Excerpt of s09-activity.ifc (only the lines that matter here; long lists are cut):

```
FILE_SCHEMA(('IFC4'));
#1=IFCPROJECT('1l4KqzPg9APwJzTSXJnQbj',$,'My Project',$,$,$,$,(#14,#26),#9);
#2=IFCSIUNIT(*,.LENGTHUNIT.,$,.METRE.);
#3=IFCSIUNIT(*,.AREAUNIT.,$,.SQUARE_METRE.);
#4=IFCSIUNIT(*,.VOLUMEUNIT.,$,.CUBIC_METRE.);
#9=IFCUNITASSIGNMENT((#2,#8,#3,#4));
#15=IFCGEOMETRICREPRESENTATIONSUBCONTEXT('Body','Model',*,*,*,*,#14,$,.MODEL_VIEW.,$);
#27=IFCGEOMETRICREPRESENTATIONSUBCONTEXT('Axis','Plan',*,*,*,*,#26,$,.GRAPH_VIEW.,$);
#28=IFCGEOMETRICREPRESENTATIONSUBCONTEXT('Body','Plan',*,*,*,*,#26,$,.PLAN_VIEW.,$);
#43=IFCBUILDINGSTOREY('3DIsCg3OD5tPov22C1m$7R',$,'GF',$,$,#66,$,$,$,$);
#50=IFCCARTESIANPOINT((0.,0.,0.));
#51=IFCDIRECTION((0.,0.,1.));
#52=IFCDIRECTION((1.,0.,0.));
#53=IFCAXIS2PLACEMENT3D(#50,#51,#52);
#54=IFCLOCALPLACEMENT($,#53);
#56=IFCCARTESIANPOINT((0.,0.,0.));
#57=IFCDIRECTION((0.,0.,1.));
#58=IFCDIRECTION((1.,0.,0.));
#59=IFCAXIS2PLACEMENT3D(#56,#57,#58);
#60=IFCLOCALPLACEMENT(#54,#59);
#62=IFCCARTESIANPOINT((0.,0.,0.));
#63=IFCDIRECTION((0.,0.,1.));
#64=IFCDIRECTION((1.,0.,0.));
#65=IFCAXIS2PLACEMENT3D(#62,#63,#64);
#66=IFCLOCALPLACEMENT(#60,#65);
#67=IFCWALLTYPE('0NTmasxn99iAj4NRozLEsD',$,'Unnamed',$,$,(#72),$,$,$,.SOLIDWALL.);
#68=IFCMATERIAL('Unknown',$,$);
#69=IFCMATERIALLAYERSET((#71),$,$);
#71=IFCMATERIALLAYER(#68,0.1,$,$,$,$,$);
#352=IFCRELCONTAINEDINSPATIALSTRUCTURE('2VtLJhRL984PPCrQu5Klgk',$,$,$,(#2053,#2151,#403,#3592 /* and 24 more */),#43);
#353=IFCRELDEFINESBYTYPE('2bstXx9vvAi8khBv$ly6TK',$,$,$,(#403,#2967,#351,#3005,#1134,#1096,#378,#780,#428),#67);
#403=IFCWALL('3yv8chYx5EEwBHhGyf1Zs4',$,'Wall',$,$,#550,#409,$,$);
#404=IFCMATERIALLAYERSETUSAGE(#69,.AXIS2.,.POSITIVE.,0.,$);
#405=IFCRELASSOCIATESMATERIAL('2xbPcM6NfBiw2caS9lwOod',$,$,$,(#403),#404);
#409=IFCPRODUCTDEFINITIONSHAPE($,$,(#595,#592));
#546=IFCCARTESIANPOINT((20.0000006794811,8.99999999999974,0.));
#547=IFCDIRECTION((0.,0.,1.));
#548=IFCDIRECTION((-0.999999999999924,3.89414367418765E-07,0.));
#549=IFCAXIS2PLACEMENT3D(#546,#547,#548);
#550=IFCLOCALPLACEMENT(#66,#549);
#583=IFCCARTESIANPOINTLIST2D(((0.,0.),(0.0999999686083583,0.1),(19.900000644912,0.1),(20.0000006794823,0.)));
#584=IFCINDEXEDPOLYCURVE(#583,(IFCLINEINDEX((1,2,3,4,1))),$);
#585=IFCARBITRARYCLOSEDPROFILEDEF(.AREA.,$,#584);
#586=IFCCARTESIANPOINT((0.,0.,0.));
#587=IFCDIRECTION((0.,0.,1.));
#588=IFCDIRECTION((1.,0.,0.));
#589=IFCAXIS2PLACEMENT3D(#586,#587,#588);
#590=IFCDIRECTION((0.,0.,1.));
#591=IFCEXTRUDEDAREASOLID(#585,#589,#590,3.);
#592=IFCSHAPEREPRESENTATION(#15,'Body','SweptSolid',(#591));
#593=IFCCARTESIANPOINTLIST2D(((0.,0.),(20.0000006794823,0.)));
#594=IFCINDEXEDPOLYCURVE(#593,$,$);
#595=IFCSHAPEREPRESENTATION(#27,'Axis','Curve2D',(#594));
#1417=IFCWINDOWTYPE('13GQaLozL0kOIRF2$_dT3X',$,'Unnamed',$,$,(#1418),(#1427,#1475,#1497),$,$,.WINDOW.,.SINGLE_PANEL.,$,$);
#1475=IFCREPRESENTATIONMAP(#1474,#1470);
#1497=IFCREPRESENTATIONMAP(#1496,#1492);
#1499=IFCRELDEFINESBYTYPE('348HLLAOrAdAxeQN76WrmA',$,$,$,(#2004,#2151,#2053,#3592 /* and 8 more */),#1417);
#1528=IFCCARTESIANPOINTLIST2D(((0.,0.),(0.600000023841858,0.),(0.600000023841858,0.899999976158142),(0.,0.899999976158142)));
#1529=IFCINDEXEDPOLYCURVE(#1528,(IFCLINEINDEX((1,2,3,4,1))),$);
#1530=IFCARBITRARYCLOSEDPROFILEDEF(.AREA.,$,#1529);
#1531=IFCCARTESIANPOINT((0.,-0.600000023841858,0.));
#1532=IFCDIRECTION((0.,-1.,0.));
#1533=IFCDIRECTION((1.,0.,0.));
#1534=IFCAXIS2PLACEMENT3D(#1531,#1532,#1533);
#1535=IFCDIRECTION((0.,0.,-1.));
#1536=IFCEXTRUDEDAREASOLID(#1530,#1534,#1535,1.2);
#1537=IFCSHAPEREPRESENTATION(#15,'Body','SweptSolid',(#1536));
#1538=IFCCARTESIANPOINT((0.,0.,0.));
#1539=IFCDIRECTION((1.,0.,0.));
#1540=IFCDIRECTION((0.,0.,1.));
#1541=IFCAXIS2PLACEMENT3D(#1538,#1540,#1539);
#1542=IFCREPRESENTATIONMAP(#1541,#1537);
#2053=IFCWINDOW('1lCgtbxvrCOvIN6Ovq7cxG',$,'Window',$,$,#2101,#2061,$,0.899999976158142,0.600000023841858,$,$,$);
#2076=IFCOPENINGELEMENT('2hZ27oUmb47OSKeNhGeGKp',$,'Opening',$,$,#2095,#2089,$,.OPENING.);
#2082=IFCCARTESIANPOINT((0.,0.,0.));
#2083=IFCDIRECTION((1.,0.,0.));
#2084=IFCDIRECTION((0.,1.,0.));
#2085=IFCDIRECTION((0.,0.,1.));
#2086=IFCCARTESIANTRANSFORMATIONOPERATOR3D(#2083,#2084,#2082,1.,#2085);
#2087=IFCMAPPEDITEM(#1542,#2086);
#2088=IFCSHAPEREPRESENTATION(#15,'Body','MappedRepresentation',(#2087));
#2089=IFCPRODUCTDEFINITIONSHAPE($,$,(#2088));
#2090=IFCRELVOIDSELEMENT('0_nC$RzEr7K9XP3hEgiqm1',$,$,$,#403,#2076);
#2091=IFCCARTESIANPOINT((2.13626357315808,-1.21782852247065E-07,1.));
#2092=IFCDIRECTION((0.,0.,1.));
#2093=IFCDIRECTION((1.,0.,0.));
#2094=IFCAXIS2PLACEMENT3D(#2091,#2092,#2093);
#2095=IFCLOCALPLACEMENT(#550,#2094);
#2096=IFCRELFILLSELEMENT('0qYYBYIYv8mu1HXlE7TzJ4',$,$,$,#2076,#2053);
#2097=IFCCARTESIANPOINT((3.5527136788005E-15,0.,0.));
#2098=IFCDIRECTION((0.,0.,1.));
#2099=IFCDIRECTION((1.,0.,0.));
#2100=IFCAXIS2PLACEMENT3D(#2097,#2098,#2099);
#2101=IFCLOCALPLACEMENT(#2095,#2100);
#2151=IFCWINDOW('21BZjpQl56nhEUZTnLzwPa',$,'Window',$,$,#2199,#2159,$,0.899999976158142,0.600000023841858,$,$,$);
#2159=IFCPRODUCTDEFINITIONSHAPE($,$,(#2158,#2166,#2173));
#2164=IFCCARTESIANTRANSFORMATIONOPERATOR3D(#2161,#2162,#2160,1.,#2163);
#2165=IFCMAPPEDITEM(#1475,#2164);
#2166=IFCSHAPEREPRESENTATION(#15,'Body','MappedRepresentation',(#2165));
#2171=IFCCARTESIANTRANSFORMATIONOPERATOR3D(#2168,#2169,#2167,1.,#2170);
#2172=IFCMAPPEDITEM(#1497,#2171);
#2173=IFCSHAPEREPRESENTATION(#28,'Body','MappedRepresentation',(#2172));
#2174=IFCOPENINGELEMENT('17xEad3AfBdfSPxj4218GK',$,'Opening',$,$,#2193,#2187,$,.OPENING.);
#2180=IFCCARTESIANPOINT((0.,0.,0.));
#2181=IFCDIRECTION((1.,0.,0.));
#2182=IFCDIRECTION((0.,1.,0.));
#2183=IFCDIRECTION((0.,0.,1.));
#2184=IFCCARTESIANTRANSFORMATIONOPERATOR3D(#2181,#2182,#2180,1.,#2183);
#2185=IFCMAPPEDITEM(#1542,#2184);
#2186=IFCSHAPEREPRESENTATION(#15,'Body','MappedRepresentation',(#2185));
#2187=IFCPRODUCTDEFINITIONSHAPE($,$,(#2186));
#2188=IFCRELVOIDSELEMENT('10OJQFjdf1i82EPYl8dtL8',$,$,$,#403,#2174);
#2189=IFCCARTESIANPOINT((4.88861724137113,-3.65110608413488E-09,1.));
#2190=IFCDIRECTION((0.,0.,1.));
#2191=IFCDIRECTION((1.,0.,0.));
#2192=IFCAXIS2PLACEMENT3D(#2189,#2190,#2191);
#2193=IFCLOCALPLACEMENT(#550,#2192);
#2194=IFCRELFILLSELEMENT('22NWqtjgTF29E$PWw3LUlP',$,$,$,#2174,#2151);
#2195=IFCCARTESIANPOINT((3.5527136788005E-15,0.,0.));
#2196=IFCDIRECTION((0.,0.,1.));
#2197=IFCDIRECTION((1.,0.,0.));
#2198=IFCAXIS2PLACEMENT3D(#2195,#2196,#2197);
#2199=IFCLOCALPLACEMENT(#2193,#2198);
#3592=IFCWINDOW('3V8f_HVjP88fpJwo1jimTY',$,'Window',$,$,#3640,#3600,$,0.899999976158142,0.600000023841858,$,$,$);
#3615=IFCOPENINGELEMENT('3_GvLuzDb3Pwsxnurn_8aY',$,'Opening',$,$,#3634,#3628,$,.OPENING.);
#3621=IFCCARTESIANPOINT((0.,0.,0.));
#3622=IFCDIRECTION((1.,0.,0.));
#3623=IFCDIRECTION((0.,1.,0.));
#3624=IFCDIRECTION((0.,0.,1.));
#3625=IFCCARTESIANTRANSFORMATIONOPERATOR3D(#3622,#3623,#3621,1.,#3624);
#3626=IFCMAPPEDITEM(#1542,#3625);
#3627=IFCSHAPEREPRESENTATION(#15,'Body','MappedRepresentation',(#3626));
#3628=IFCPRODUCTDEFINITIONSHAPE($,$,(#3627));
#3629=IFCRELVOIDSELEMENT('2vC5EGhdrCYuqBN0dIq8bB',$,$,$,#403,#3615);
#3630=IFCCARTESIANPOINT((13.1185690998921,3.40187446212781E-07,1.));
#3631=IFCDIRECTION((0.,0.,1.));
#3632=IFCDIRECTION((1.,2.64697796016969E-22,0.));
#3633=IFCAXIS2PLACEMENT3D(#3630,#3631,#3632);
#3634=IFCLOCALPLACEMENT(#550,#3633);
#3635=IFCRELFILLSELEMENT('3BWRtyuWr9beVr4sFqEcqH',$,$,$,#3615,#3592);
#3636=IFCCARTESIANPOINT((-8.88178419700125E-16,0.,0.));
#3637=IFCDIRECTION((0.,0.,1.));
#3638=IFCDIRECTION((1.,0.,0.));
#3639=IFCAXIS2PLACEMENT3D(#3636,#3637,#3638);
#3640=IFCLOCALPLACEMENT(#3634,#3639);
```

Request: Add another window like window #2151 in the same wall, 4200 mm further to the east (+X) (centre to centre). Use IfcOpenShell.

```python
import ifcopenshell
import ifcopenshell.api.feature
import ifcopenshell.api.geometry
import ifcopenshell.api.root
import ifcopenshell.geom
import ifcopenshell.util.element
import ifcopenshell.util.placement
import ifcopenshell.util.shape

model = ifcopenshell.open("s09-activity.ifc")
settings = ifcopenshell.geom.settings()


def volume(element):
    """Net volume in cubic metres, openings subtracted."""
    shape = ifcopenshell.geom.create_shape(settings, element)
    return ifcopenshell.util.shape.get_volume(shape.geometry)


window = model.by_id(2151)
opening = window.FillsVoids[0].RelatingOpeningElement
wall = opening.VoidsElements[0].RelatingBuildingElement
before = volume(wall)
shift = ifcopenshell.util.placement.get_local_placement(wall.ObjectPlacement)[:3, 0] * -4.2

# copy_class copies the void relationship, type, container and properties, but no geometry.
new_opening = ifcopenshell.api.root.copy_class(model, product=opening)
new_opening.Representation = ifcopenshell.util.element.copy_deep(
    model, opening.Representation, exclude=["IfcGeometricRepresentationContext", "IfcRepresentationMap"]
)
new_window = ifcopenshell.api.root.copy_class(model, product=window)
new_window.Representation = ifcopenshell.util.element.copy_deep(
    model, window.Representation, exclude=["IfcGeometricRepresentationContext", "IfcRepresentationMap"]
)
ifcopenshell.api.feature.add_filling(model, opening=new_opening, element=new_window)

for old, new in ((opening, new_opening), (window, new_window)):
    matrix = ifcopenshell.util.placement.get_local_placement(old.ObjectPlacement)
    matrix[:3, 3] += shift
    ifcopenshell.api.geometry.edit_object_placement(model, product=new, matrix=matrix, is_si=False)

after = volume(wall)

print(f"wall volume {before:.3f} -> {after:.3f} m3")

model.write("s09-activity_edited.ifc")
```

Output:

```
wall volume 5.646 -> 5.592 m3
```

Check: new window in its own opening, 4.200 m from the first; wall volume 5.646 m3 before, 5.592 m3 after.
